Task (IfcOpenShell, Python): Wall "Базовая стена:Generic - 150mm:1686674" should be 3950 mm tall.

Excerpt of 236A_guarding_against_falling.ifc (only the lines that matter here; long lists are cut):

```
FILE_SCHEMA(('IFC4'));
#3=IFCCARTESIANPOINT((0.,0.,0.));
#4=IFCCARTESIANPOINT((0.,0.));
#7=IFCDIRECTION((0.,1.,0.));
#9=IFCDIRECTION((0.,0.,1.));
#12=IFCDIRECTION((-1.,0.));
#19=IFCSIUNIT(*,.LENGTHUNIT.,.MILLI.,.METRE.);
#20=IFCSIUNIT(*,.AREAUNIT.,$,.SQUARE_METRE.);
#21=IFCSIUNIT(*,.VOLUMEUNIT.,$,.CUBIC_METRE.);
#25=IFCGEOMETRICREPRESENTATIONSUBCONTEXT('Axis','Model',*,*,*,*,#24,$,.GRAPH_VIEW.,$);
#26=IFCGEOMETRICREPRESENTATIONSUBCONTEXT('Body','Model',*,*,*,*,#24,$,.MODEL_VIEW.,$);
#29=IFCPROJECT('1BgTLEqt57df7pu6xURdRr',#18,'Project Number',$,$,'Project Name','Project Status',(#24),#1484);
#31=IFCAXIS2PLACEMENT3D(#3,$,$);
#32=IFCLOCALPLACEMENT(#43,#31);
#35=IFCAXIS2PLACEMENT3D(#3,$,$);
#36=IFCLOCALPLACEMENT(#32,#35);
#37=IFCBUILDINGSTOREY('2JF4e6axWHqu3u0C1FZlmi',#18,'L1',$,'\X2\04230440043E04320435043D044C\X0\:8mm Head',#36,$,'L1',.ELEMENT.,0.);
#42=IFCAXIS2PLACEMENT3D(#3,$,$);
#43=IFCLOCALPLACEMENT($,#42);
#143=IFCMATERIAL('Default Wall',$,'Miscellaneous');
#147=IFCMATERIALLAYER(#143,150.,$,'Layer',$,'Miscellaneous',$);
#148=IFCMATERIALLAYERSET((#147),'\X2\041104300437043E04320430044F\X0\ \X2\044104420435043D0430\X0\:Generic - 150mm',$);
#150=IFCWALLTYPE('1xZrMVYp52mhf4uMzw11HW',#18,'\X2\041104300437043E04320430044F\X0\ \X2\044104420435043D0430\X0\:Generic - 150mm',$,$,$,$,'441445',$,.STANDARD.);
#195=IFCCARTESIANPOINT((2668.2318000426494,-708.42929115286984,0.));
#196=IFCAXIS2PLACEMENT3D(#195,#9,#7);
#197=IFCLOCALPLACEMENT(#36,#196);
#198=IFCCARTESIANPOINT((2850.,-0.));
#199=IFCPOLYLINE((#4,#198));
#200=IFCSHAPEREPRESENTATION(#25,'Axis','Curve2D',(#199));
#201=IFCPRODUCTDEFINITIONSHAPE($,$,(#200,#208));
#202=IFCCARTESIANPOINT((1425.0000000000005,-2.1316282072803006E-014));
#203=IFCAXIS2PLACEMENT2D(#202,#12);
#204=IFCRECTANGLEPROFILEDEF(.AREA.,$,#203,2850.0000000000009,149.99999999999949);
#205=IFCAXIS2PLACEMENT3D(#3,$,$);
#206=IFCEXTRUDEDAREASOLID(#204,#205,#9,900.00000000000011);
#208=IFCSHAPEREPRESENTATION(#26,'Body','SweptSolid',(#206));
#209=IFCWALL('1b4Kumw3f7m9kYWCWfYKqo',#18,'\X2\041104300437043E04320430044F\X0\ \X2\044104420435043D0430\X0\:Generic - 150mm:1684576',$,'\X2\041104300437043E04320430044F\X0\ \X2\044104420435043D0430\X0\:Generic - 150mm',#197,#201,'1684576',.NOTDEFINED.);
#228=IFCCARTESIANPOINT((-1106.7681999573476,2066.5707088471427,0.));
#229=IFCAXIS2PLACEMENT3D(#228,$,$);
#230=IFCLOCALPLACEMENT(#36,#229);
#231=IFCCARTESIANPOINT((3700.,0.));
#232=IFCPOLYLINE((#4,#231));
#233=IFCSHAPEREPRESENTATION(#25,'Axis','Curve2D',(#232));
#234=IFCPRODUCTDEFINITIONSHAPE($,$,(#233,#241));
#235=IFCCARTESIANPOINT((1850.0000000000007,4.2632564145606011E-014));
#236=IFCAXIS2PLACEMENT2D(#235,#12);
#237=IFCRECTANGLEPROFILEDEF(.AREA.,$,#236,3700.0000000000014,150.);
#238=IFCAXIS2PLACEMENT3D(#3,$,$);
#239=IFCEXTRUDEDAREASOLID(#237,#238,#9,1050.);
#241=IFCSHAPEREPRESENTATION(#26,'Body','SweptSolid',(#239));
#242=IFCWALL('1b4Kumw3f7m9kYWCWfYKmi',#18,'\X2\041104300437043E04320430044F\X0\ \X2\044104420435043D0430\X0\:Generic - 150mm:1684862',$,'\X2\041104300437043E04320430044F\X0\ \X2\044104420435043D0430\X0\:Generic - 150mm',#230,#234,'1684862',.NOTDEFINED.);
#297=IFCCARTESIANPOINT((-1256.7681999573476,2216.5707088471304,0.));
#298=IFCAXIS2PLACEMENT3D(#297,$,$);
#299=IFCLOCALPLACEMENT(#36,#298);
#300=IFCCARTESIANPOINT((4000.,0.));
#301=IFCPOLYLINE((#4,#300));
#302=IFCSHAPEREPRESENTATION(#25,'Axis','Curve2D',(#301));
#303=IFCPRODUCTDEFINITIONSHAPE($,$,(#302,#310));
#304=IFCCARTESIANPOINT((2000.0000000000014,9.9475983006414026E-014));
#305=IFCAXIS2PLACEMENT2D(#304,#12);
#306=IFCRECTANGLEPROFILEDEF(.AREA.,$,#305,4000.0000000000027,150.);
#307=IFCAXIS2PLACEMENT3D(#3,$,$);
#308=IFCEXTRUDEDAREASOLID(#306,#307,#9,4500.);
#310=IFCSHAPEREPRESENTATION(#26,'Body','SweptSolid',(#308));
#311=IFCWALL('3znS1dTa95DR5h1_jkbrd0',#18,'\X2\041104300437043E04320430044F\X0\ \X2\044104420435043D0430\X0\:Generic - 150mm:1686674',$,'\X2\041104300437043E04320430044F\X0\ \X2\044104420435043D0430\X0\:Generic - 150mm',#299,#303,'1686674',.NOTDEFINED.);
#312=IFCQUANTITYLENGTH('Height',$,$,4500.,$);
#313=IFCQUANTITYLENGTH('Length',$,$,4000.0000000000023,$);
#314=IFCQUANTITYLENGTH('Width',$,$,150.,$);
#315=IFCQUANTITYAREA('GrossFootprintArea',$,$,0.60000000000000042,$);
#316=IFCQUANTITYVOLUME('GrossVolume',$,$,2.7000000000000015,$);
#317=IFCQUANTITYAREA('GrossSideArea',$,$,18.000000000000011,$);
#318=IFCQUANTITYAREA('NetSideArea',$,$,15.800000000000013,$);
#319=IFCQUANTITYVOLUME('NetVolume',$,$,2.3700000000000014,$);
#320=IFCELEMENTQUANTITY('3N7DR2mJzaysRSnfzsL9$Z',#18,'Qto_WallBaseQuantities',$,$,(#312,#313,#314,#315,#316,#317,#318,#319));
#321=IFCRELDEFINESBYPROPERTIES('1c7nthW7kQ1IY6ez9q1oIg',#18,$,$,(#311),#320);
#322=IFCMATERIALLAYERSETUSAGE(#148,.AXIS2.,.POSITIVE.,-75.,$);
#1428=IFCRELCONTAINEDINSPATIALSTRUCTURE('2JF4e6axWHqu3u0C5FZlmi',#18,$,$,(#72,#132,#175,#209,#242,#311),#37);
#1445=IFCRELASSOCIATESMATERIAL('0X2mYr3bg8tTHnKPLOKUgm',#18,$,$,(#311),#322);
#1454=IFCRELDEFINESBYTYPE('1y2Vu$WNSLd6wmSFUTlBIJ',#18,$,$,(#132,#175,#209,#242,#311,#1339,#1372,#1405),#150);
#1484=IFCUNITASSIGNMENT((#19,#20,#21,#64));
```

```python
import ifcopenshell
import ifcopenshell.api.pset
import ifcopenshell.geom
import ifcopenshell.util.element
import ifcopenshell.util.representation
import ifcopenshell.util.shape
import ifcopenshell.util.unit

model = ifcopenshell.open("236A_guarding_against_falling.ifc")
unit_scale = ifcopenshell.util.unit.calculate_unit_scale(model)
area_scale = ifcopenshell.util.unit.calculate_unit_scale(model, "AREAUNIT")
volume_scale = ifcopenshell.util.unit.calculate_unit_scale(model, "VOLUMEUNIT")
settings = ifcopenshell.geom.settings()


def volume(element):
    """Net volume in cubic metres, openings subtracted."""
    shape = ifcopenshell.geom.create_shape(settings, element)
    return ifcopenshell.util.shape.get_volume(shape.geometry)


wall = model.by_guid("3znS1dTa95DR5h1_jkbrd0")
before = volume(wall)

body = ifcopenshell.util.representation.get_representation(wall, "Model", "Body")
solid = body.Items[0]
old_height = solid.Depth
solid.Depth = 3950.0
after = volume(wall)
thickness = 0.15  # wall thickness in metres

# Update the stored height, areas and volumes.
qto = model.by_id(ifcopenshell.util.element.get_pset(wall, "Qto_WallBaseQuantities", should_inherit=False)["id"])
ifcopenshell.api.pset.edit_qto(model, qto=qto, properties={
    "Height": solid.Depth,
    "GrossVolume": ifcopenshell.util.element.get_pset(wall, "Qto_WallBaseQuantities", "GrossVolume") * solid.Depth / old_height,
    "GrossSideArea": ifcopenshell.util.element.get_pset(wall, "Qto_WallBaseQuantities", "GrossSideArea") * solid.Depth / old_height,
    "NetSideArea": after / thickness / area_scale,
    "NetVolume": after / volume_scale,
})

print(f"height {old_height:g} -> {solid.Depth:g}, volume {before:.3f} -> {after:.3f} m3")

model.write("236A_guarding_against_falling_rev.ifc")
```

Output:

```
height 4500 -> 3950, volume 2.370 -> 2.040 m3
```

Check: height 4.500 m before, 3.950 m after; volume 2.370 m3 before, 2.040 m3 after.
